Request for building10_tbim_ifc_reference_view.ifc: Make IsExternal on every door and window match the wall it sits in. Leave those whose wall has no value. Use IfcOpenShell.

First a look at what the model holds.

```python
import ifcopenshell
import ifcopenshell.util.element

model = ifcopenshell.open("building10_tbim_ifc_reference_view.ifc")
print(model.schema)
seen = {}
for e in model.by_type("IfcDoor") + model.by_type("IfcWindow"):
    if not e.FillsVoids:
        continue
    host = e.FillsVoids[0].RelatingOpeningElement.VoidsElements[0].RelatingBuildingElement
    own = ifcopenshell.util.element.get_pset(e, f"Pset_{e.is_a()[3:].removesuffix('StandardCase')}Common", "IsExternal")
    wall = ifcopenshell.util.element.get_pset(host, "Pset_WallCommon", "IsExternal")
    seen[e.is_a(), own, wall] = seen.get((e.is_a(), own, wall), 0) + 1
for (cls, own, wall), count in sorted(seen.items(), key=str):
    print(count, cls, "IsExternal:", own, "| host wall:", wall)
```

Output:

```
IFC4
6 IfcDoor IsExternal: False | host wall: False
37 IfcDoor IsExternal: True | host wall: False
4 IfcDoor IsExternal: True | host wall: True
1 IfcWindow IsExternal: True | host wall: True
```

```python
import ifcopenshell
import ifcopenshell.api.pset
import ifcopenshell.util.element

model = ifcopenshell.open("building10_tbim_ifc_reference_view.ifc")

count = 0
for ifc_class, pset_name in (("IfcDoor", "Pset_DoorCommon"), ("IfcWindow", "Pset_WindowCommon")):
    for e in model.by_type(ifc_class):
        if not e.FillsVoids:
            continue
        host = e.FillsVoids[0].RelatingOpeningElement.VoidsElements[0].RelatingBuildingElement
        external = ifcopenshell.util.element.get_pset(host, "Pset_WallCommon", "IsExternal")
        if external is None or ifcopenshell.util.element.get_pset(e, pset_name, "IsExternal") == external:
            continue
        pset = ifcopenshell.api.pset.add_pset(model, product=e, name=pset_name)
        ifcopenshell.api.pset.edit_pset(model, pset=pset, properties={"IsExternal": external})
        count += 1

print(count, "updated")

model.write("building10_tbim_ifc_reference_view_edited.ifc")
```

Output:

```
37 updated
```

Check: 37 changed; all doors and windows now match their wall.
